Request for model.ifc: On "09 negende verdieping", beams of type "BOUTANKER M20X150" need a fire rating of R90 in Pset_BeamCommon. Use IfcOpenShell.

First a look at what the model holds.

```python
import ifcopenshell
import ifcopenshell.util.element

model = ifcopenshell.open("model.ifc")
print(model.schema)
storey = next(s for s in model.by_type("IfcBuildingStorey") if s.Name == "09 negende verdieping")
beams = [e for e in ifcopenshell.util.element.get_decomposition(storey) if e.is_a("IfcBeam")]
seen = {}
for e in beams:
    element_type = ifcopenshell.util.element.get_type(e)
    key = (element_type.Name if element_type != e and element_type else None, ifcopenshell.util.element.get_pset(e, "Pset_BeamCommon", "FireRating"))
    seen[key] = seen.get(key, 0) + 1
for (name, value), count in sorted(seen.items(), key=str):
    print(count, "x", name, "|", value)
```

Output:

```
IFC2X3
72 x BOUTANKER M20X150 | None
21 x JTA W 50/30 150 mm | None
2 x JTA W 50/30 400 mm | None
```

```python
import ifcopenshell
import ifcopenshell.api.pset
import ifcopenshell.util.element

model = ifcopenshell.open("model.ifc")

storey = next(s for s in model.by_type("IfcBuildingStorey") if s.Name == "09 negende verdieping")
beams = [e for e in ifcopenshell.util.element.get_decomposition(storey) if e.is_a("IfcBeam")]

count = 0
for e in beams:
    element_type = ifcopenshell.util.element.get_type(e)
    if element_type in (None, e) or element_type.Name != "BOUTANKER M20X150":
        continue
    # add_pset returns the element's existing set when there is one.
    pset = ifcopenshell.api.pset.add_pset(model, product=e, name="Pset_BeamCommon")
    ifcopenshell.api.pset.edit_pset(model, pset=pset, properties={"FireRating": "R90"})
    count += 1

print(count, "beams updated")

model.write("model-out.ifc")
```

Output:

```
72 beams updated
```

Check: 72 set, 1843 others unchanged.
